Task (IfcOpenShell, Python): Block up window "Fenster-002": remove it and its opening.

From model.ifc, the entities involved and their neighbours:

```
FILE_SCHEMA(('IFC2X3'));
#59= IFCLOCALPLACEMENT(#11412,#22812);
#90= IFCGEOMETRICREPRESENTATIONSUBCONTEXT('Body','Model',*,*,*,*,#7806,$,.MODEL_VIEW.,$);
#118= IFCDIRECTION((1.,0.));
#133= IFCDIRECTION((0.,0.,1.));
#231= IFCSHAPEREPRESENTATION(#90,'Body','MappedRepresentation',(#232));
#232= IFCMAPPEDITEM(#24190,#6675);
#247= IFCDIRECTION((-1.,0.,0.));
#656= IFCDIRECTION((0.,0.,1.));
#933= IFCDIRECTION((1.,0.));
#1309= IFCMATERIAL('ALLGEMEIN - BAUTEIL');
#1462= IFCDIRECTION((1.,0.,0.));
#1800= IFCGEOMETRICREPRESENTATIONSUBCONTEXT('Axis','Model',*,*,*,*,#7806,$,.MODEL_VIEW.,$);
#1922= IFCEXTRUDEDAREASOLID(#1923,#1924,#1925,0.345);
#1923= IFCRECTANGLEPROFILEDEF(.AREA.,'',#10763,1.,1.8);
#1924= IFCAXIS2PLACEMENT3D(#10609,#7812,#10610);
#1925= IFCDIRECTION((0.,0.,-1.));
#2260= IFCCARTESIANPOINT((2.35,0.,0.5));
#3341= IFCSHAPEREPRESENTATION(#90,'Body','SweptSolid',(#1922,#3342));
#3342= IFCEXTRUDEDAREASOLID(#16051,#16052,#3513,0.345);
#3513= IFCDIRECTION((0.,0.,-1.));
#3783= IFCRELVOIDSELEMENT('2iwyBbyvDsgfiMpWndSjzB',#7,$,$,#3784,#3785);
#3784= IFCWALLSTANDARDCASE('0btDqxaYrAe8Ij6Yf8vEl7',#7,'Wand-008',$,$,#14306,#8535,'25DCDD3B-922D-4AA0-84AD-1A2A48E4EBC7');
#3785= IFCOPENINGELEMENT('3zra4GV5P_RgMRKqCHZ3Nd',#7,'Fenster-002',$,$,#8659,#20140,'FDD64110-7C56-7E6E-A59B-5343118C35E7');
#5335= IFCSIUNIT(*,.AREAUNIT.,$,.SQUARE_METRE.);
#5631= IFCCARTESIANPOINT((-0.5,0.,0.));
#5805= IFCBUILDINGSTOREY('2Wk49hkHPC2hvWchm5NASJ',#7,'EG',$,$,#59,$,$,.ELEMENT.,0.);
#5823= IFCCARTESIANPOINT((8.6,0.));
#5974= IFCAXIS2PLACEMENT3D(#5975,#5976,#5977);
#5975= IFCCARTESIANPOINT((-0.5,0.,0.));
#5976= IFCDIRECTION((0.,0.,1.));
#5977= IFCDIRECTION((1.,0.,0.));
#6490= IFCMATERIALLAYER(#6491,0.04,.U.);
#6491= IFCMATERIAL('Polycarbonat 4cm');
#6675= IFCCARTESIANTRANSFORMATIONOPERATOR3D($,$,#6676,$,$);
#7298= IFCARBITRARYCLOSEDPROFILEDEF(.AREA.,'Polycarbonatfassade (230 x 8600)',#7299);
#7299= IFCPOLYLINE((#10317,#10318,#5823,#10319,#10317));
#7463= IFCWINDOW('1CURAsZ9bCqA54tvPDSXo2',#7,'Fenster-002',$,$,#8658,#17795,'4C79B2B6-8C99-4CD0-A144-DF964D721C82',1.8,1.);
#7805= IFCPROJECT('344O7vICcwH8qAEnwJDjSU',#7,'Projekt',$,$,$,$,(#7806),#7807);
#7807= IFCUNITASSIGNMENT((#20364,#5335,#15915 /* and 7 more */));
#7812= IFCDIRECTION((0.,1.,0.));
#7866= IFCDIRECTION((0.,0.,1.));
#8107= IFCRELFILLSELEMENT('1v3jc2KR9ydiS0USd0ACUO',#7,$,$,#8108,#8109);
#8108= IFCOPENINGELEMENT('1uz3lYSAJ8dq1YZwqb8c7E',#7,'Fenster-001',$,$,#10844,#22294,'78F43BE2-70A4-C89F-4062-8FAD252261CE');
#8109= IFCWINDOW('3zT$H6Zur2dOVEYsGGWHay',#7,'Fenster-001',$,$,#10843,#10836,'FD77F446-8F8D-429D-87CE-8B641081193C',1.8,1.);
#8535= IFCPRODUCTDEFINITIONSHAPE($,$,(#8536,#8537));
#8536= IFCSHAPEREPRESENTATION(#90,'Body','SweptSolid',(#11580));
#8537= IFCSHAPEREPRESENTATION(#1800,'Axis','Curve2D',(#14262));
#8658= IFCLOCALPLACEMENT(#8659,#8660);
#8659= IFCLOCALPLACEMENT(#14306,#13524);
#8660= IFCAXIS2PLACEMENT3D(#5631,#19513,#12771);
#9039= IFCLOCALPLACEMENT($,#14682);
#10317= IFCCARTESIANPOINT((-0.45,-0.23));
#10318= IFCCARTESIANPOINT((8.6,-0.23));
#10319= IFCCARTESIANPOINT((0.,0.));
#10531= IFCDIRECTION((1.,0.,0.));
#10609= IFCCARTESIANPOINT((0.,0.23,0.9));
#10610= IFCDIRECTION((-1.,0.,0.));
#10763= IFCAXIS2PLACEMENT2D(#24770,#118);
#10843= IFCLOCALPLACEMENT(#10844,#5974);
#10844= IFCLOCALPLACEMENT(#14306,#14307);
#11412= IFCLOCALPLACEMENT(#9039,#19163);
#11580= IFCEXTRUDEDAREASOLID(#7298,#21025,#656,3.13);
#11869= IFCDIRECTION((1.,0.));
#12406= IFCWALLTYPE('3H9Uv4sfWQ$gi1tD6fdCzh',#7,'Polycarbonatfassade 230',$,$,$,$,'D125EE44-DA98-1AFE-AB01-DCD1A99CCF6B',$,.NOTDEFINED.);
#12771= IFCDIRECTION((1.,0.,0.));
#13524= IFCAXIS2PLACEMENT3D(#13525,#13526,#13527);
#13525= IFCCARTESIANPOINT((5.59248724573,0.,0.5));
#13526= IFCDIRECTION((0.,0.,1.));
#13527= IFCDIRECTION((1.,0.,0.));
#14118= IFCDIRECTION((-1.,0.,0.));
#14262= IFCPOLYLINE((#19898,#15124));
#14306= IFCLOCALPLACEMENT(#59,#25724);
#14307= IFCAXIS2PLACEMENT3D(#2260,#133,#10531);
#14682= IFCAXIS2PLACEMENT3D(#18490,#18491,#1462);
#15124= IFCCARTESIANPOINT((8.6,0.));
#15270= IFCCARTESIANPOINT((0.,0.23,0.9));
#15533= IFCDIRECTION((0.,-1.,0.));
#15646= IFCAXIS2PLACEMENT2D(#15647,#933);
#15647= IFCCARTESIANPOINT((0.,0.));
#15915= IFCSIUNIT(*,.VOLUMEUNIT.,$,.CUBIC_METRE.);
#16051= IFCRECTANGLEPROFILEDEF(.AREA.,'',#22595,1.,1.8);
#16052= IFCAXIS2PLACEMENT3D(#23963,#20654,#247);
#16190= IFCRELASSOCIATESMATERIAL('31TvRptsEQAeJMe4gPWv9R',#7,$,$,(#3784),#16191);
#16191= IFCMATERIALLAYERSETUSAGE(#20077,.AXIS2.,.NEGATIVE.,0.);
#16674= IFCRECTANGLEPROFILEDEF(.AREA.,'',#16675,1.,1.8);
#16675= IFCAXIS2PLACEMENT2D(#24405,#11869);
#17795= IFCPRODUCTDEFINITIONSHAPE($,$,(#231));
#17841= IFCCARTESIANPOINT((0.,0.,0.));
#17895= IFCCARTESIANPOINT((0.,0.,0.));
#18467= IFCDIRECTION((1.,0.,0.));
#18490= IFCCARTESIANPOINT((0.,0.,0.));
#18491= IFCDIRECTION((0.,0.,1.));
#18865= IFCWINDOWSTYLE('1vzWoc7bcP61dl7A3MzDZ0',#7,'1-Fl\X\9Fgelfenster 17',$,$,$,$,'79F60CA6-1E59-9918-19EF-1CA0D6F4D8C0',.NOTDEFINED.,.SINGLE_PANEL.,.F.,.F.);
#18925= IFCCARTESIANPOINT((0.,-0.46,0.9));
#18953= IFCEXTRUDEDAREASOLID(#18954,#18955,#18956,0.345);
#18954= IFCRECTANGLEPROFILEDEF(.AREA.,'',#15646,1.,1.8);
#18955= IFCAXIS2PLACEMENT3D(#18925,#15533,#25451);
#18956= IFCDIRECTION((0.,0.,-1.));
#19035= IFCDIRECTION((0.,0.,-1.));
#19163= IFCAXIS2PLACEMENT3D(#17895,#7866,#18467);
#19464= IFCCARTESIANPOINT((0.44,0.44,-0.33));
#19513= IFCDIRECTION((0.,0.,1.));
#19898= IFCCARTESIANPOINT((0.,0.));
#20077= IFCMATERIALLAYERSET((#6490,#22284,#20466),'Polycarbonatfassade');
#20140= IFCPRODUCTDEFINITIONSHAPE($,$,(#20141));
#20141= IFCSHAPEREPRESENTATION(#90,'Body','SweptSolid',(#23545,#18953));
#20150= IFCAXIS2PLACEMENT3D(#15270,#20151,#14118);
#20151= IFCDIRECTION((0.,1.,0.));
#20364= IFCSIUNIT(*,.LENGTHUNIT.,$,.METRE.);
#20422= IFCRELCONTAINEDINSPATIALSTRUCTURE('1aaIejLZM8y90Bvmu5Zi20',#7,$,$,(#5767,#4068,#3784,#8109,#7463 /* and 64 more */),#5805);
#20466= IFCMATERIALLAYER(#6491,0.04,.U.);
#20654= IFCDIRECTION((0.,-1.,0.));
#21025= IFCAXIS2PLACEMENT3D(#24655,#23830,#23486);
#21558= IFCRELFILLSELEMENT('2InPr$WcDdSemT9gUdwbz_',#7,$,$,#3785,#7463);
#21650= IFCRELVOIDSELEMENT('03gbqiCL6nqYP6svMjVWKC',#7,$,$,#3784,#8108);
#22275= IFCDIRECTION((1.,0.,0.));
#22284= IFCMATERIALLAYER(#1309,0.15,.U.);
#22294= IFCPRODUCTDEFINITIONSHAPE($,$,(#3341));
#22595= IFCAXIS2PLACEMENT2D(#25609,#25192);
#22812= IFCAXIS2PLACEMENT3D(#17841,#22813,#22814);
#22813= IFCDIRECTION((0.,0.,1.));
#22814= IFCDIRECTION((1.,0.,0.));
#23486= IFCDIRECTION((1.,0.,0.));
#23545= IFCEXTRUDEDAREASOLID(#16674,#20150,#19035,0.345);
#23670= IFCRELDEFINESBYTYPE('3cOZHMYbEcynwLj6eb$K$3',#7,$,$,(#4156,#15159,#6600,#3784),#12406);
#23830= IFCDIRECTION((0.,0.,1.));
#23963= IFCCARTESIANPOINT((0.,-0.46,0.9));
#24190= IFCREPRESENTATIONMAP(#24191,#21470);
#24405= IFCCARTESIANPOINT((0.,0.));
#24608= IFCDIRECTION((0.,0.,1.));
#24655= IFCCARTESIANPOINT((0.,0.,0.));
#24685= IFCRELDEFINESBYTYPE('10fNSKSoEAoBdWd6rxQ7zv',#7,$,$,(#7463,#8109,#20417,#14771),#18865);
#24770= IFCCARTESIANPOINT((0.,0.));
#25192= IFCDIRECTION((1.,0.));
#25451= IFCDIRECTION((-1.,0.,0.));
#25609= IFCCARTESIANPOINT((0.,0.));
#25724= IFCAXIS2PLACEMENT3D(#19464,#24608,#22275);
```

```python
import ifcopenshell
import ifcopenshell.api.feature
import ifcopenshell.api.root
import ifcopenshell.geom
import ifcopenshell.util.shape

model = ifcopenshell.open("model.ifc")
settings = ifcopenshell.geom.settings()


def volume(element):
    """Net volume in cubic metres, openings subtracted."""
    shape = ifcopenshell.geom.create_shape(settings, element)
    return ifcopenshell.util.shape.get_volume(shape.geometry)


window = model.by_id(7463)
opening = window.FillsVoids[0].RelatingOpeningElement
wall = opening.VoidsElements[0].RelatingBuildingElement
before = volume(wall)

ifcopenshell.api.root.remove_product(model, product=window)
ifcopenshell.api.feature.remove_feature(model, feature=opening)

after = volume(wall)

print(f"wall volume {before:.3f} -> {after:.3f} m3")

model.write("model_rev.ifc")
```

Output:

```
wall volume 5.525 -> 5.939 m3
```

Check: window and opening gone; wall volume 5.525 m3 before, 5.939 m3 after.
